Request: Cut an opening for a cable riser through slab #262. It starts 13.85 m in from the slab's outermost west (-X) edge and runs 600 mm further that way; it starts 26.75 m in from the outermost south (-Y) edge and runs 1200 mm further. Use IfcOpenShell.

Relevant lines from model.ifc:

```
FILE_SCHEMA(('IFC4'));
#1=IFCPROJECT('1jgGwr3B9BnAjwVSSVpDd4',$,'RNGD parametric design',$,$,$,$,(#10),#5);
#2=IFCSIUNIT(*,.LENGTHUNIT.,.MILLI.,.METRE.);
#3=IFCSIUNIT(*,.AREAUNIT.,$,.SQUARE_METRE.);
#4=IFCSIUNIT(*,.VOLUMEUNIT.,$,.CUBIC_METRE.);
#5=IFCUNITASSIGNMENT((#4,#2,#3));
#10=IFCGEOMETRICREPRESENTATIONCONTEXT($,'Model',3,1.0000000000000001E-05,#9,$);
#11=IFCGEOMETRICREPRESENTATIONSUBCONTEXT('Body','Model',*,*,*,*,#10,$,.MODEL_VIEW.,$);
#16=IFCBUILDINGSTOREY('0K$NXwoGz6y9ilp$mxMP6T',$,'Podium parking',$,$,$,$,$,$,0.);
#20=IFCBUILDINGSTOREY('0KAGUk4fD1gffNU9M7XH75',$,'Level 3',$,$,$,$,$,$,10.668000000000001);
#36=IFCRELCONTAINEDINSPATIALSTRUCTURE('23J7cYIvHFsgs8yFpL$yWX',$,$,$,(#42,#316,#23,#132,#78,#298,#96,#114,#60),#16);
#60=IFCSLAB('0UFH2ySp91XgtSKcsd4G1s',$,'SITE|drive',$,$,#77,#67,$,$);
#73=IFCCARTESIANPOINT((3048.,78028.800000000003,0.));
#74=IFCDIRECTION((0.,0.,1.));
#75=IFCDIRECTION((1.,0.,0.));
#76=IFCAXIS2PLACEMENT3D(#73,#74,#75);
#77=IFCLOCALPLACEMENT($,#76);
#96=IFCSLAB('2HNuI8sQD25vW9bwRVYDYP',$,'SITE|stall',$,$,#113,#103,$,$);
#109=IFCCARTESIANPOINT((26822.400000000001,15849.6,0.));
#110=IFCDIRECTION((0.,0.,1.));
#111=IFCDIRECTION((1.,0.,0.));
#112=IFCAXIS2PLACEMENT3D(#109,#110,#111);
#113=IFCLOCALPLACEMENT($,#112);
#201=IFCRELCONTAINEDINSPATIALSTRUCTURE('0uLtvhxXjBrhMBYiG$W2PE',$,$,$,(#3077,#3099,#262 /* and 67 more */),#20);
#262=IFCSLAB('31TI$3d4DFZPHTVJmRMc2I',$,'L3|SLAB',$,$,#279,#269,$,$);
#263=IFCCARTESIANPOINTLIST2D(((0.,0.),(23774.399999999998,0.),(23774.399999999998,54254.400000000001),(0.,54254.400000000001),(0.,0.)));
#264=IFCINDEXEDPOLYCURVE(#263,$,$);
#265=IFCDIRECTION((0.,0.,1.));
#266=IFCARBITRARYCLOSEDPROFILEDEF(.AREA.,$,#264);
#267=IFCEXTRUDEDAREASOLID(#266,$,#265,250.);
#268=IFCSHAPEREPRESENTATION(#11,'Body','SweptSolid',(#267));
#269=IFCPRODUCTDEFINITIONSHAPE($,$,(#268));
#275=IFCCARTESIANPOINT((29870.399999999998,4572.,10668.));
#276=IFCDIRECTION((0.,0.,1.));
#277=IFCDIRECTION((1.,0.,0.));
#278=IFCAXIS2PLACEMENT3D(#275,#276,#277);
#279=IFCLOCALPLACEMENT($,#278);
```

```python
import numpy as np
import ifcopenshell
import ifcopenshell.api.feature
import ifcopenshell.api.geometry
import ifcopenshell.api.root
import ifcopenshell.geom
import ifcopenshell.util.placement
import ifcopenshell.util.representation
import ifcopenshell.util.shape
import ifcopenshell.util.unit

model = ifcopenshell.open("model.ifc")
unit_scale = ifcopenshell.util.unit.calculate_unit_scale(model)
settings = ifcopenshell.geom.settings()


def volume(element):
    """Net volume in cubic metres, openings subtracted."""
    shape = ifcopenshell.geom.create_shape(settings, element)
    return ifcopenshell.util.shape.get_volume(shape.geometry)


slab = model.by_guid("31TI$3d4DFZPHTVJmRMc2I")
before = volume(slab)

# Extent in the slab's own axes, in metres. The edges named are its -X and -Y sides.
slab_shape = ifcopenshell.geom.create_shape(settings, slab)
vertices = ifcopenshell.util.shape.get_vertices(slab_shape.geometry)
x_min, y_min, bottom = vertices.min(axis=0)
top = vertices[:, 2].max()

opening = ifcopenshell.api.root.create_entity(model, ifc_class="IfcOpeningElement", name="Cable riser opening", predefined_type="OPENING")
context = ifcopenshell.util.representation.get_context(model, "Model", "Body", "MODEL_VIEW")
width, depth = 0.6, 1.2
outline = [(0.0, 0.0), (width, 0.0), (width, depth), (0.0, depth), (0.0, 0.0)]
# Overshoot both faces by 50 mm so the cut is clean.
shape = ifcopenshell.api.geometry.add_slab_representation(
    model, context=context, depth=top - bottom + 0.1, polyline=outline
)
ifcopenshell.api.geometry.assign_representation(model, product=opening, representation=shape)

matrix = ifcopenshell.util.placement.get_local_placement(slab.ObjectPlacement)
matrix[:, 3] = matrix @ np.append(np.array([x_min + 13.85, y_min + 26.75, bottom - 0.05]) / unit_scale, 1.0)
ifcopenshell.api.geometry.edit_object_placement(model, product=opening, matrix=matrix, is_si=False)
ifcopenshell.api.feature.add_feature(model, feature=opening, element=slab)

after = volume(slab)

print(f"slab volume {before:.3f} -> {after:.3f} m3")

model.write("model-out.ifc")
```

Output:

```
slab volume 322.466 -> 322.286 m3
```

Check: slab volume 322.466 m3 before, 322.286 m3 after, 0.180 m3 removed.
